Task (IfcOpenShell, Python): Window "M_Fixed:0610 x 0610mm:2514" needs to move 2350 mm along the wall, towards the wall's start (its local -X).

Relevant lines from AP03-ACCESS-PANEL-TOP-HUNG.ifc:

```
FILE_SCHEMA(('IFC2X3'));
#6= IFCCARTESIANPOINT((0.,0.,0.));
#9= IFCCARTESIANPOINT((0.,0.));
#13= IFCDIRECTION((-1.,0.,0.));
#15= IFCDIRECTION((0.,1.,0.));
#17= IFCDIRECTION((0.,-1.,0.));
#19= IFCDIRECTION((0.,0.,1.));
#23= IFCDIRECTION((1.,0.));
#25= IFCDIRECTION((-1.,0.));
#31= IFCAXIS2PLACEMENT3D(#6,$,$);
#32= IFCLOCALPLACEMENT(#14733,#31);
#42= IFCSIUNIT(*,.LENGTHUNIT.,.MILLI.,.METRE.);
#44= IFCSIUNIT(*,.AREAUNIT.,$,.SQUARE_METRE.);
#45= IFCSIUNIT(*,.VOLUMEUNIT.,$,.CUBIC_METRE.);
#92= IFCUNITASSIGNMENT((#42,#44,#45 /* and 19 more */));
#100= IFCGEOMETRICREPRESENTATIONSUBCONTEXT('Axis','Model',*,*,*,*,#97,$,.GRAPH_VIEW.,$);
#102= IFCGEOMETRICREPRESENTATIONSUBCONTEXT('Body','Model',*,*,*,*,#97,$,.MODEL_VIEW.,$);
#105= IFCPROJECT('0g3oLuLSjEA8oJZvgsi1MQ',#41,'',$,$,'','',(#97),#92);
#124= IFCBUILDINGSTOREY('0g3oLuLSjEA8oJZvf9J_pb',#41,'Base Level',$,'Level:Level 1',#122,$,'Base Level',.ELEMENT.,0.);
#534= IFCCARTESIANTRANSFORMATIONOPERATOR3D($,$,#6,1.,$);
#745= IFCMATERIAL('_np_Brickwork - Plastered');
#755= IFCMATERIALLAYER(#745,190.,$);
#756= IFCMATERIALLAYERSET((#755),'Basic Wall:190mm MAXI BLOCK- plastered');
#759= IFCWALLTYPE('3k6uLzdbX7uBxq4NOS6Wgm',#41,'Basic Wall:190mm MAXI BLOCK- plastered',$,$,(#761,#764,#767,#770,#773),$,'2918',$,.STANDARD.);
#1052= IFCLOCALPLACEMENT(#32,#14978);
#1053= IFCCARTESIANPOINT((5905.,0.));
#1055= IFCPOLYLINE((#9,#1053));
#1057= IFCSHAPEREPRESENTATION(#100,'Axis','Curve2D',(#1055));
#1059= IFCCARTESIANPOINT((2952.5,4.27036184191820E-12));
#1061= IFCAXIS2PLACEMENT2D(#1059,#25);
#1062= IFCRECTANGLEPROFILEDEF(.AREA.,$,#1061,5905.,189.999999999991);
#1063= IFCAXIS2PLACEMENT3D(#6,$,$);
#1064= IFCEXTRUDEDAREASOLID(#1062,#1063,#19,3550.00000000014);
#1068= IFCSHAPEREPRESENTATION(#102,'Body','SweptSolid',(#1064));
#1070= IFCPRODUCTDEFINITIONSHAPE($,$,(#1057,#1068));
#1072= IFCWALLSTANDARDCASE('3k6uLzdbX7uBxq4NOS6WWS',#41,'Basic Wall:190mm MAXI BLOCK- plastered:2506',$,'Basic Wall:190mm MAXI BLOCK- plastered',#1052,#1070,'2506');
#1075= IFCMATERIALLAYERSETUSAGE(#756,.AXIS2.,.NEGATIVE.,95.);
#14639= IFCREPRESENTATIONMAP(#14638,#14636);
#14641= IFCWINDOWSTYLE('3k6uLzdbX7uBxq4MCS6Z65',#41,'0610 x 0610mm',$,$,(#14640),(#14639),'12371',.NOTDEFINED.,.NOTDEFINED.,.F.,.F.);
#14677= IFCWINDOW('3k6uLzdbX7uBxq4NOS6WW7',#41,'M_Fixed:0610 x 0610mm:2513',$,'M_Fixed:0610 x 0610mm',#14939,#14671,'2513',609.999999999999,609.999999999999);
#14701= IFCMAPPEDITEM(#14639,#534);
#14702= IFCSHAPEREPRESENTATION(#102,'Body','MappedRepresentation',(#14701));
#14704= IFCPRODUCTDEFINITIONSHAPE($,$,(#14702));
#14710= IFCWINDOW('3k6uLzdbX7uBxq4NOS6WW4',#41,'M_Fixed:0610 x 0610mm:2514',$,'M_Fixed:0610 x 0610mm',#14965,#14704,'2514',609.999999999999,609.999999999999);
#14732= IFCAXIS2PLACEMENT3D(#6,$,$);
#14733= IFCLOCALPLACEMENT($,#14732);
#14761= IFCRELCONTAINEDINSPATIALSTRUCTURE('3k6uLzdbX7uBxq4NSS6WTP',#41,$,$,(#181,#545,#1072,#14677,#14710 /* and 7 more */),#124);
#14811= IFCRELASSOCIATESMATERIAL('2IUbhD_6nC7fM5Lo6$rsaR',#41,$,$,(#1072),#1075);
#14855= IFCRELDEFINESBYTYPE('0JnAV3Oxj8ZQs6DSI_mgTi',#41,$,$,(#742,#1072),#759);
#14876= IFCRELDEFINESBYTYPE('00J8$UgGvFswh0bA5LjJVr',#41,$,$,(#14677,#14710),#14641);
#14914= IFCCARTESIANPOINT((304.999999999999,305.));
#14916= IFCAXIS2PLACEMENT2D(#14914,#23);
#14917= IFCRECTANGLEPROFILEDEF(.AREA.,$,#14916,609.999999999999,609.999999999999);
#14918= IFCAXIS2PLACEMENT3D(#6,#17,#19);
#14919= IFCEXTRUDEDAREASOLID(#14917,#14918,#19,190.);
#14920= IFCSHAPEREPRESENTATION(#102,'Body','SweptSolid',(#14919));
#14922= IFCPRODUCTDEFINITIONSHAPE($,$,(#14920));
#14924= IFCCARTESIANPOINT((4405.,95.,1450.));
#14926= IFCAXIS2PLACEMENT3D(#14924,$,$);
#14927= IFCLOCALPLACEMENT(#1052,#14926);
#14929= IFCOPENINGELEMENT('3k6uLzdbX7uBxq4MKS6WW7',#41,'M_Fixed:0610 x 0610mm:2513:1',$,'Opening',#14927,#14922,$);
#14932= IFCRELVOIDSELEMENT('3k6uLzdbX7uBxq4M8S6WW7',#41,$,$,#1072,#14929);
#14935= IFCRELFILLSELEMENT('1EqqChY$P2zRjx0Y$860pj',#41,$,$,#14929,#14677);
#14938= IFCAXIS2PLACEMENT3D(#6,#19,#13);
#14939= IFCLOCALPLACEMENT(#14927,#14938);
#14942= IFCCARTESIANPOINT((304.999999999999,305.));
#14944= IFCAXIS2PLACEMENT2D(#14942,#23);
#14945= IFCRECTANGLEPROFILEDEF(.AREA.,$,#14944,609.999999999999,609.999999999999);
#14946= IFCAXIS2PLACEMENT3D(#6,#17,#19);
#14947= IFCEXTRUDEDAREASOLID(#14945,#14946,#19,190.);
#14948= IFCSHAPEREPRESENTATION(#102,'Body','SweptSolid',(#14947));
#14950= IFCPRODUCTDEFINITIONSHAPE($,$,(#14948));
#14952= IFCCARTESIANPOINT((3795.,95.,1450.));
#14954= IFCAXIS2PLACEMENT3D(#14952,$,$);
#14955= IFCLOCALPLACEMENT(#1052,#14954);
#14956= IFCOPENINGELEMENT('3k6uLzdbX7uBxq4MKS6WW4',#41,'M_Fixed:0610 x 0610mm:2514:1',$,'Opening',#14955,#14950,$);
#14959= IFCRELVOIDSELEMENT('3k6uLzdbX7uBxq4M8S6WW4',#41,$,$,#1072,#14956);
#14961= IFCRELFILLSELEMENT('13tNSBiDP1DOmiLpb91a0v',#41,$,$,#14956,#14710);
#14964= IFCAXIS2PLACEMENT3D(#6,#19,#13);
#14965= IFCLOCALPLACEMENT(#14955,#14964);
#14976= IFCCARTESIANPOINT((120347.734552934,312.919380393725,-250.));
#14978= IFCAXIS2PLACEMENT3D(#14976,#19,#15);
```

```python
import ifcopenshell
import ifcopenshell.api.geometry
import ifcopenshell.util.placement
import ifcopenshell.util.unit

model = ifcopenshell.open("AP03-ACCESS-PANEL-TOP-HUNG.ifc")
unit_scale = ifcopenshell.util.unit.calculate_unit_scale(model)

window = model.by_guid("3k6uLzdbX7uBxq4NOS6WW4")
opening = window.FillsVoids[0].RelatingOpeningElement
wall = opening.VoidsElements[0].RelatingBuildingElement

wall_matrix = ifcopenshell.util.placement.get_local_placement(wall.ObjectPlacement)
shift = wall_matrix[:3, 0] * -2.35 / unit_scale
before = ifcopenshell.util.placement.get_local_placement(window.ObjectPlacement)[:3, 3].copy()

# The window is placed relative to its opening, so it follows when the opening moves.
matrix = ifcopenshell.util.placement.get_local_placement(opening.ObjectPlacement)
matrix[:3, 3] += shift
ifcopenshell.api.geometry.edit_object_placement(
    model, product=opening, matrix=matrix, is_si=False, should_transform_children=True
)

after = ifcopenshell.util.placement.get_local_placement(window.ObjectPlacement)[:3, 3]
print("window moved by", (after - before).round(3) + 0.0)

model.write("AP03-ACCESS-PANEL-TOP-HUNG_v2.ifc")
```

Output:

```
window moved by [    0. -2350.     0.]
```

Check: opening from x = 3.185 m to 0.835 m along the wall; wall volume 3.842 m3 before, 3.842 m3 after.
